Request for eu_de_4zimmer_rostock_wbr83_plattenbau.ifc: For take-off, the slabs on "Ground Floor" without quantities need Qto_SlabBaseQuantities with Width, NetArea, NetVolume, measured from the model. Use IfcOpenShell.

First a look at what the model holds.

```python
import ifcopenshell
import ifcopenshell.util.element
import ifcopenshell.util.unit

model = ifcopenshell.open("eu_de_4zimmer_rostock_wbr83_plattenbau.ifc")
print(model.schema)
for unit_type in ("LENGTHUNIT", "AREAUNIT", "VOLUMEUNIT"):
    print(unit_type, ifcopenshell.util.unit.calculate_unit_scale(model, unit_type))
storey = next(s for s in model.by_type("IfcBuildingStorey") if s.Name == "Ground Floor")
slabs = [e for e in ifcopenshell.util.element.get_decomposition(storey) if e.is_a("IfcSlab")]
for e in sorted(slabs, key=lambda e: e.id()):
    print(e.id(), e.is_a(), e.Name, list(ifcopenshell.util.element.get_psets(e, qtos_only=True)), sep=" | ")
```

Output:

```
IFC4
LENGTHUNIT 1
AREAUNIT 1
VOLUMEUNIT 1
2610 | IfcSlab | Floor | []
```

```python
import ifcopenshell
import ifcopenshell.api.pset
import ifcopenshell.geom
import ifcopenshell.util.element
import ifcopenshell.util.shape
import ifcopenshell.util.unit

model = ifcopenshell.open("eu_de_4zimmer_rostock_wbr83_plattenbau.ifc")
unit_scale = ifcopenshell.util.unit.calculate_unit_scale(model)
area_scale = ifcopenshell.util.unit.calculate_unit_scale(model, "AREAUNIT")
volume_scale = ifcopenshell.util.unit.calculate_unit_scale(model, "VOLUMEUNIT")
settings = ifcopenshell.geom.settings()

storey = next(s for s in model.by_type("IfcBuildingStorey") if s.Name == "Ground Floor")
slabs = [e for e in ifcopenshell.util.element.get_decomposition(storey) if e.is_a("IfcSlab")]

for e in sorted(slabs, key=lambda e: e.id()):
    if ifcopenshell.util.element.get_psets(e, qtos_only=True, should_inherit=False):
        continue
    # Geometry comes back in metres, in the element's own axes.
    shape = ifcopenshell.geom.create_shape(settings, e)
    values = {
        "Width": ifcopenshell.util.shape.get_z(shape.geometry) / unit_scale,
        "NetArea": ifcopenshell.util.shape.get_footprint_area(shape.geometry) / area_scale,
        "NetVolume": ifcopenshell.util.shape.get_volume(shape.geometry) / volume_scale,
    }
    qto = ifcopenshell.api.pset.add_qto(model, product=e, name="Qto_SlabBaseQuantities")
    ifcopenshell.api.pset.edit_qto(model, qto=qto, properties=values)
    print(e.id(), {k: round(v, 3) for k, v in values.items()})

model.write("eu_de_4zimmer_rostock_wbr83_plattenbau_v2.ifc")
```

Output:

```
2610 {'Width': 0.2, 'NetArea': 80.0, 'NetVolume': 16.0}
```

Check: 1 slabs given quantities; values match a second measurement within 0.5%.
